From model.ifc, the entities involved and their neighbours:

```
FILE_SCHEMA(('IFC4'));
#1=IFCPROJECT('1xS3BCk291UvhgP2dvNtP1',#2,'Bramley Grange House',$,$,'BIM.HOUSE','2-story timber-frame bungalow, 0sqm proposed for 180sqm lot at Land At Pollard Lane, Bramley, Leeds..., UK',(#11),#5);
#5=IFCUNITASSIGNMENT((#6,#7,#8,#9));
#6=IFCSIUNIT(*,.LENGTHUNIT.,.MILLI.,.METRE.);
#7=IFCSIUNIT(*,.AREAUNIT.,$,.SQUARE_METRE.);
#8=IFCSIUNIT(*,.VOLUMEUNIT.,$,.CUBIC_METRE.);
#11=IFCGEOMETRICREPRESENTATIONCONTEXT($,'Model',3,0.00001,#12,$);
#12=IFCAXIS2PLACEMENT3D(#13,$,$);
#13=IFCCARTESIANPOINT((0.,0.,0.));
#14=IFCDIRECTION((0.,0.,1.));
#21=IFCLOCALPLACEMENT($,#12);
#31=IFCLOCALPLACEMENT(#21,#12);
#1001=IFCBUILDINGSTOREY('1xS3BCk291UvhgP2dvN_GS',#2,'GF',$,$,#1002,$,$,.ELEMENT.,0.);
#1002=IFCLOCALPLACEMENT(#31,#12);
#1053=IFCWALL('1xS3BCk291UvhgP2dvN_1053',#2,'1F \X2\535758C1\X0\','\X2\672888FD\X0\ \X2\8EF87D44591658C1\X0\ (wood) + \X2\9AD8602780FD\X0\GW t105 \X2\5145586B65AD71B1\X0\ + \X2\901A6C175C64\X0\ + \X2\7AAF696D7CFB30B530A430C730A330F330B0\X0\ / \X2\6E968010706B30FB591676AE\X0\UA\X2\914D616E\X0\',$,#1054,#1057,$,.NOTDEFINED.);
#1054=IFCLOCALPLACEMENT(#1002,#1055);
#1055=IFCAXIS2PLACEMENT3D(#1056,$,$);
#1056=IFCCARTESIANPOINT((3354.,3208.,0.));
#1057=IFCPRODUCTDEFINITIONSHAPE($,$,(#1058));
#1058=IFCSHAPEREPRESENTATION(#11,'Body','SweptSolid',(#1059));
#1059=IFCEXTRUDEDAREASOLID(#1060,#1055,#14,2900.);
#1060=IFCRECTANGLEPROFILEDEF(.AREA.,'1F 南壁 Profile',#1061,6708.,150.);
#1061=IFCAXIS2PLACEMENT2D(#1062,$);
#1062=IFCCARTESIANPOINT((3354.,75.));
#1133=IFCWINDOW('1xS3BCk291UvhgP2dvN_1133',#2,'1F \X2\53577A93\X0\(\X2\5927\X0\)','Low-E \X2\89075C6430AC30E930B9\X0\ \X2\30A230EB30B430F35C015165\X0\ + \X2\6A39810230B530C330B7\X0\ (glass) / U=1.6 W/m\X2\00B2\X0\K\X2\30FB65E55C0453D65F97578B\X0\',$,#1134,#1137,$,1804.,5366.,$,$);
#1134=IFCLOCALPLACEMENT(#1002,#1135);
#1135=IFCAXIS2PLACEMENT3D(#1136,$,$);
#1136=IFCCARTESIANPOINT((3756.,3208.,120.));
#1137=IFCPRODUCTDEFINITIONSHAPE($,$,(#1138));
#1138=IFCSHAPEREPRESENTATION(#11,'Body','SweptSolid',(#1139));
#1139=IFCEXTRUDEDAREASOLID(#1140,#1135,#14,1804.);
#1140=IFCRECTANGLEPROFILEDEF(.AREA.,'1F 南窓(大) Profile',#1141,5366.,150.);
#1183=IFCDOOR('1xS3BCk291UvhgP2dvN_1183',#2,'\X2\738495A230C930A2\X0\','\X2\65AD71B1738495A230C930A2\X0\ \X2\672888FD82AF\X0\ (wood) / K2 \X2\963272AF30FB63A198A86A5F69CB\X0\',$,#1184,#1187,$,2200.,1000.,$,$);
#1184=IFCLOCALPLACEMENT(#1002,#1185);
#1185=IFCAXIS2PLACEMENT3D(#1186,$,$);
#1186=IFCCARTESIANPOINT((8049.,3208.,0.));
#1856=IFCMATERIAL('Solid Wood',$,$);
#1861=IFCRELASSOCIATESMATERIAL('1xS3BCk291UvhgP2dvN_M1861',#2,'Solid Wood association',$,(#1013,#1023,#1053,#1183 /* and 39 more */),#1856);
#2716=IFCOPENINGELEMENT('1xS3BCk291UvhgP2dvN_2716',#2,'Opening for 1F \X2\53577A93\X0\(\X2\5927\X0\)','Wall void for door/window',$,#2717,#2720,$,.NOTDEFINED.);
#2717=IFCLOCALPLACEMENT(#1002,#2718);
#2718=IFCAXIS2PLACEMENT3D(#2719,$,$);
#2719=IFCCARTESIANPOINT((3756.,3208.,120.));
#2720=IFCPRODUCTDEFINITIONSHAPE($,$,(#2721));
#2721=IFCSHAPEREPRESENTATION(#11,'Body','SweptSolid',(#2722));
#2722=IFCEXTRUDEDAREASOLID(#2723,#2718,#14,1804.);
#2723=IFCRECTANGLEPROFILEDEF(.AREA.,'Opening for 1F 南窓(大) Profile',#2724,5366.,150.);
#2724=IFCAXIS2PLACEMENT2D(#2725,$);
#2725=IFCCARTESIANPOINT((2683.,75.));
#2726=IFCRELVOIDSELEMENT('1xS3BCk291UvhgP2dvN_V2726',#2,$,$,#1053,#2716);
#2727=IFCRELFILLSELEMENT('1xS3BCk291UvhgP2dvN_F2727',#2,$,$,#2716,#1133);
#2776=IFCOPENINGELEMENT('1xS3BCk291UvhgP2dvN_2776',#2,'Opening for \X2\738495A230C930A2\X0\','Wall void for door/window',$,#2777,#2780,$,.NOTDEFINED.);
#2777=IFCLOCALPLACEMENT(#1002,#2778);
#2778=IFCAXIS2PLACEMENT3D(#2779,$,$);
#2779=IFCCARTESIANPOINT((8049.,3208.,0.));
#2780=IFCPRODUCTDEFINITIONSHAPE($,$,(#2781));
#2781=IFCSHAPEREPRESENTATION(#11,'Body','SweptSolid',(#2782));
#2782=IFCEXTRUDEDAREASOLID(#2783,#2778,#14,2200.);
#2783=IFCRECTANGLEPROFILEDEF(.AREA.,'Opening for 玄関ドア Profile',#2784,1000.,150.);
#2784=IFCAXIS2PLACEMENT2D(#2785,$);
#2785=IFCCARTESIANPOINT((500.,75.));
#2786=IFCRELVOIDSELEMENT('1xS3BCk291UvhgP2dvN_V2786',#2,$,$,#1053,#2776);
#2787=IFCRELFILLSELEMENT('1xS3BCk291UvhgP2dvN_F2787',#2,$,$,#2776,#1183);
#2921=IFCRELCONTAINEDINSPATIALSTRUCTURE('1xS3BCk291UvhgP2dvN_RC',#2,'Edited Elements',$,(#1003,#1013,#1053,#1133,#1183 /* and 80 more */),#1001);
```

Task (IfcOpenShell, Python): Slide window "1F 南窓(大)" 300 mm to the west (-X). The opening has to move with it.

```python
import ifcopenshell
import ifcopenshell.api.geometry
import ifcopenshell.util.placement

model = ifcopenshell.open("model.ifc")

window = model.by_guid("1xS3BCk291UvhgP2dvN_1133")
opening = window.FillsVoids[0].RelatingOpeningElement
wall = opening.VoidsElements[0].RelatingBuildingElement

wall_matrix = ifcopenshell.util.placement.get_local_placement(wall.ObjectPlacement)
shift = wall_matrix[:3, 0] * -300.0
before = ifcopenshell.util.placement.get_local_placement(window.ObjectPlacement)[:3, 3].copy()

# The window is not placed relative to its opening, so move both.
for product in (opening, window):
    matrix = ifcopenshell.util.placement.get_local_placement(product.ObjectPlacement)
    matrix[:3, 3] += shift
    ifcopenshell.api.geometry.edit_object_placement(model, product=product, matrix=matrix, is_si=False)

after = ifcopenshell.util.placement.get_local_placement(window.ObjectPlacement)[:3, 3]
print("window moved by", (after - before).round(3) + 0.0)

model.write("model-out.ifc")
```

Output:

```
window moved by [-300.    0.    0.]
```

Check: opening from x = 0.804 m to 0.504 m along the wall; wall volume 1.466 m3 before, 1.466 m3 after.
